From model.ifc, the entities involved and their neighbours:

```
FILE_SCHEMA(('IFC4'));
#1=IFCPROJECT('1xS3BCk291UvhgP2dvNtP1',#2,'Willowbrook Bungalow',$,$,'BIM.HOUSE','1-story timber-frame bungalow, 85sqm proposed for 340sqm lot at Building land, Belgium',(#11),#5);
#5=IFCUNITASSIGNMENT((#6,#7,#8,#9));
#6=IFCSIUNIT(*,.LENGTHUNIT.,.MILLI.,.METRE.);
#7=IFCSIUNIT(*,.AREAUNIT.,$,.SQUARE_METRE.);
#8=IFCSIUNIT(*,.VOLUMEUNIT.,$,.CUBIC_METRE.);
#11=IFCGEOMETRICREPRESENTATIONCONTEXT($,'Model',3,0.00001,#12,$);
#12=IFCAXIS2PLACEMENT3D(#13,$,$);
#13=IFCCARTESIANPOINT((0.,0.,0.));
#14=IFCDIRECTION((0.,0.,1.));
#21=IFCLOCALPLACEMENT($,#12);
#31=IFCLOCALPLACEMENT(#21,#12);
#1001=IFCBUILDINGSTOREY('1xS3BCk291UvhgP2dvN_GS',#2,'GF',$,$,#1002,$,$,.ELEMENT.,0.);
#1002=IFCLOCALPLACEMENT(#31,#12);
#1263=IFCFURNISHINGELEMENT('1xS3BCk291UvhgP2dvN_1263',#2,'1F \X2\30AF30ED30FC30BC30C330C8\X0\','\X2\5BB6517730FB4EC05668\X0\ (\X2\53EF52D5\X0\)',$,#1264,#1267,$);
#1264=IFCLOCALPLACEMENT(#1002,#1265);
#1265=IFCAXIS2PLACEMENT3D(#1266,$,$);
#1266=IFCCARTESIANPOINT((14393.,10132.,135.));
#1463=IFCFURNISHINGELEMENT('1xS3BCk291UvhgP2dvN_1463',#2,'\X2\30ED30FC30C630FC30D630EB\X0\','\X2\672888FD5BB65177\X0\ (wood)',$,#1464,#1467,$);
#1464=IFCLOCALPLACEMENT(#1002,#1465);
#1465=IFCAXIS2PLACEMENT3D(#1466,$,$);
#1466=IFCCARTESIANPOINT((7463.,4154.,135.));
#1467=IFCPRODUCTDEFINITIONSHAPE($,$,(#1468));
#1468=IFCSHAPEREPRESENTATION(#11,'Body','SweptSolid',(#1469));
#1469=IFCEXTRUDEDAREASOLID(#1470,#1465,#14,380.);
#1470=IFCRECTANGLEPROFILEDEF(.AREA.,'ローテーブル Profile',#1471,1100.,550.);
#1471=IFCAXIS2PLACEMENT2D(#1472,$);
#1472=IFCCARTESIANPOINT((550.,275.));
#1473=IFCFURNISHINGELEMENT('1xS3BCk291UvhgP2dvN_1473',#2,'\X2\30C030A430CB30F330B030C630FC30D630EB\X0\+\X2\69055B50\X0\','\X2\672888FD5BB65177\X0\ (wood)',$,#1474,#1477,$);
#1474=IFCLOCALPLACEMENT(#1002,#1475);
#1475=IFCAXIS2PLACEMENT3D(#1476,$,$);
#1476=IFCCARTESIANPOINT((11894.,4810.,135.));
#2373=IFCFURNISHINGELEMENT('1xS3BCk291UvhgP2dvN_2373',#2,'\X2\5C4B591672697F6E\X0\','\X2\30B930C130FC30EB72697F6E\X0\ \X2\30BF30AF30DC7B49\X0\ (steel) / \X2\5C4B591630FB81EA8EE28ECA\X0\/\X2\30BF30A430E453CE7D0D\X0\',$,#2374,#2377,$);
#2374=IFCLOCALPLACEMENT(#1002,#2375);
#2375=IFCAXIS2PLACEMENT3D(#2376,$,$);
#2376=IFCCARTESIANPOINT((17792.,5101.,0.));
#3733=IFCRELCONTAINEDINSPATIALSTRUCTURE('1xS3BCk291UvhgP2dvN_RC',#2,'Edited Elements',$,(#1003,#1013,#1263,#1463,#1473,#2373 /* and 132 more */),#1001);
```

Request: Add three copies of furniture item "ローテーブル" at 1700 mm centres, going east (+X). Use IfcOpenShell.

```python
import numpy as np
import ifcopenshell
import ifcopenshell.api.geometry
import ifcopenshell.api.root
import ifcopenshell.util.element
import ifcopenshell.util.placement
import ifcopenshell.util.unit

model = ifcopenshell.open("model.ifc")
unit_scale = ifcopenshell.util.unit.calculate_unit_scale(model)


def reuse_history(source, copy):
    """copy_class also copies each property set's owner history, people and application; keep the originals."""
    for rel in copy.IsDefinedBy:
        if rel.is_a("IfcRelDefinesByProperties") and (history := rel.RelatingPropertyDefinition.OwnerHistory):
            rel.RelatingPropertyDefinition.OwnerHistory = source.OwnerHistory
            ifcopenshell.util.element.remove_deep2(model, history)


source = model.by_guid("1xS3BCk291UvhgP2dvN_1463")
base = ifcopenshell.util.placement.get_local_placement(source.ObjectPlacement)
step = np.array([1.0, 0.0, 0.0]) * 1.7 / unit_scale

for i in range(1, 4):
    copy = ifcopenshell.api.root.copy_class(model, product=source)
    copy.Representation = ifcopenshell.util.element.copy_deep(
        model, source.Representation, exclude=["IfcGeometricRepresentationContext", "IfcRepresentationMap"]
    )
    reuse_history(source, copy)
    matrix = base.copy()
    matrix[:3, 3] += i * step
    print("added at", matrix[:3, 3].round(3) + 0.0)
    ifcopenshell.api.geometry.edit_object_placement(model, product=copy, matrix=matrix, is_si=False)

model.write("model_rev.ifc")
```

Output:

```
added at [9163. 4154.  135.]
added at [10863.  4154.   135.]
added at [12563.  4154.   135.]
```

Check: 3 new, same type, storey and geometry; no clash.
